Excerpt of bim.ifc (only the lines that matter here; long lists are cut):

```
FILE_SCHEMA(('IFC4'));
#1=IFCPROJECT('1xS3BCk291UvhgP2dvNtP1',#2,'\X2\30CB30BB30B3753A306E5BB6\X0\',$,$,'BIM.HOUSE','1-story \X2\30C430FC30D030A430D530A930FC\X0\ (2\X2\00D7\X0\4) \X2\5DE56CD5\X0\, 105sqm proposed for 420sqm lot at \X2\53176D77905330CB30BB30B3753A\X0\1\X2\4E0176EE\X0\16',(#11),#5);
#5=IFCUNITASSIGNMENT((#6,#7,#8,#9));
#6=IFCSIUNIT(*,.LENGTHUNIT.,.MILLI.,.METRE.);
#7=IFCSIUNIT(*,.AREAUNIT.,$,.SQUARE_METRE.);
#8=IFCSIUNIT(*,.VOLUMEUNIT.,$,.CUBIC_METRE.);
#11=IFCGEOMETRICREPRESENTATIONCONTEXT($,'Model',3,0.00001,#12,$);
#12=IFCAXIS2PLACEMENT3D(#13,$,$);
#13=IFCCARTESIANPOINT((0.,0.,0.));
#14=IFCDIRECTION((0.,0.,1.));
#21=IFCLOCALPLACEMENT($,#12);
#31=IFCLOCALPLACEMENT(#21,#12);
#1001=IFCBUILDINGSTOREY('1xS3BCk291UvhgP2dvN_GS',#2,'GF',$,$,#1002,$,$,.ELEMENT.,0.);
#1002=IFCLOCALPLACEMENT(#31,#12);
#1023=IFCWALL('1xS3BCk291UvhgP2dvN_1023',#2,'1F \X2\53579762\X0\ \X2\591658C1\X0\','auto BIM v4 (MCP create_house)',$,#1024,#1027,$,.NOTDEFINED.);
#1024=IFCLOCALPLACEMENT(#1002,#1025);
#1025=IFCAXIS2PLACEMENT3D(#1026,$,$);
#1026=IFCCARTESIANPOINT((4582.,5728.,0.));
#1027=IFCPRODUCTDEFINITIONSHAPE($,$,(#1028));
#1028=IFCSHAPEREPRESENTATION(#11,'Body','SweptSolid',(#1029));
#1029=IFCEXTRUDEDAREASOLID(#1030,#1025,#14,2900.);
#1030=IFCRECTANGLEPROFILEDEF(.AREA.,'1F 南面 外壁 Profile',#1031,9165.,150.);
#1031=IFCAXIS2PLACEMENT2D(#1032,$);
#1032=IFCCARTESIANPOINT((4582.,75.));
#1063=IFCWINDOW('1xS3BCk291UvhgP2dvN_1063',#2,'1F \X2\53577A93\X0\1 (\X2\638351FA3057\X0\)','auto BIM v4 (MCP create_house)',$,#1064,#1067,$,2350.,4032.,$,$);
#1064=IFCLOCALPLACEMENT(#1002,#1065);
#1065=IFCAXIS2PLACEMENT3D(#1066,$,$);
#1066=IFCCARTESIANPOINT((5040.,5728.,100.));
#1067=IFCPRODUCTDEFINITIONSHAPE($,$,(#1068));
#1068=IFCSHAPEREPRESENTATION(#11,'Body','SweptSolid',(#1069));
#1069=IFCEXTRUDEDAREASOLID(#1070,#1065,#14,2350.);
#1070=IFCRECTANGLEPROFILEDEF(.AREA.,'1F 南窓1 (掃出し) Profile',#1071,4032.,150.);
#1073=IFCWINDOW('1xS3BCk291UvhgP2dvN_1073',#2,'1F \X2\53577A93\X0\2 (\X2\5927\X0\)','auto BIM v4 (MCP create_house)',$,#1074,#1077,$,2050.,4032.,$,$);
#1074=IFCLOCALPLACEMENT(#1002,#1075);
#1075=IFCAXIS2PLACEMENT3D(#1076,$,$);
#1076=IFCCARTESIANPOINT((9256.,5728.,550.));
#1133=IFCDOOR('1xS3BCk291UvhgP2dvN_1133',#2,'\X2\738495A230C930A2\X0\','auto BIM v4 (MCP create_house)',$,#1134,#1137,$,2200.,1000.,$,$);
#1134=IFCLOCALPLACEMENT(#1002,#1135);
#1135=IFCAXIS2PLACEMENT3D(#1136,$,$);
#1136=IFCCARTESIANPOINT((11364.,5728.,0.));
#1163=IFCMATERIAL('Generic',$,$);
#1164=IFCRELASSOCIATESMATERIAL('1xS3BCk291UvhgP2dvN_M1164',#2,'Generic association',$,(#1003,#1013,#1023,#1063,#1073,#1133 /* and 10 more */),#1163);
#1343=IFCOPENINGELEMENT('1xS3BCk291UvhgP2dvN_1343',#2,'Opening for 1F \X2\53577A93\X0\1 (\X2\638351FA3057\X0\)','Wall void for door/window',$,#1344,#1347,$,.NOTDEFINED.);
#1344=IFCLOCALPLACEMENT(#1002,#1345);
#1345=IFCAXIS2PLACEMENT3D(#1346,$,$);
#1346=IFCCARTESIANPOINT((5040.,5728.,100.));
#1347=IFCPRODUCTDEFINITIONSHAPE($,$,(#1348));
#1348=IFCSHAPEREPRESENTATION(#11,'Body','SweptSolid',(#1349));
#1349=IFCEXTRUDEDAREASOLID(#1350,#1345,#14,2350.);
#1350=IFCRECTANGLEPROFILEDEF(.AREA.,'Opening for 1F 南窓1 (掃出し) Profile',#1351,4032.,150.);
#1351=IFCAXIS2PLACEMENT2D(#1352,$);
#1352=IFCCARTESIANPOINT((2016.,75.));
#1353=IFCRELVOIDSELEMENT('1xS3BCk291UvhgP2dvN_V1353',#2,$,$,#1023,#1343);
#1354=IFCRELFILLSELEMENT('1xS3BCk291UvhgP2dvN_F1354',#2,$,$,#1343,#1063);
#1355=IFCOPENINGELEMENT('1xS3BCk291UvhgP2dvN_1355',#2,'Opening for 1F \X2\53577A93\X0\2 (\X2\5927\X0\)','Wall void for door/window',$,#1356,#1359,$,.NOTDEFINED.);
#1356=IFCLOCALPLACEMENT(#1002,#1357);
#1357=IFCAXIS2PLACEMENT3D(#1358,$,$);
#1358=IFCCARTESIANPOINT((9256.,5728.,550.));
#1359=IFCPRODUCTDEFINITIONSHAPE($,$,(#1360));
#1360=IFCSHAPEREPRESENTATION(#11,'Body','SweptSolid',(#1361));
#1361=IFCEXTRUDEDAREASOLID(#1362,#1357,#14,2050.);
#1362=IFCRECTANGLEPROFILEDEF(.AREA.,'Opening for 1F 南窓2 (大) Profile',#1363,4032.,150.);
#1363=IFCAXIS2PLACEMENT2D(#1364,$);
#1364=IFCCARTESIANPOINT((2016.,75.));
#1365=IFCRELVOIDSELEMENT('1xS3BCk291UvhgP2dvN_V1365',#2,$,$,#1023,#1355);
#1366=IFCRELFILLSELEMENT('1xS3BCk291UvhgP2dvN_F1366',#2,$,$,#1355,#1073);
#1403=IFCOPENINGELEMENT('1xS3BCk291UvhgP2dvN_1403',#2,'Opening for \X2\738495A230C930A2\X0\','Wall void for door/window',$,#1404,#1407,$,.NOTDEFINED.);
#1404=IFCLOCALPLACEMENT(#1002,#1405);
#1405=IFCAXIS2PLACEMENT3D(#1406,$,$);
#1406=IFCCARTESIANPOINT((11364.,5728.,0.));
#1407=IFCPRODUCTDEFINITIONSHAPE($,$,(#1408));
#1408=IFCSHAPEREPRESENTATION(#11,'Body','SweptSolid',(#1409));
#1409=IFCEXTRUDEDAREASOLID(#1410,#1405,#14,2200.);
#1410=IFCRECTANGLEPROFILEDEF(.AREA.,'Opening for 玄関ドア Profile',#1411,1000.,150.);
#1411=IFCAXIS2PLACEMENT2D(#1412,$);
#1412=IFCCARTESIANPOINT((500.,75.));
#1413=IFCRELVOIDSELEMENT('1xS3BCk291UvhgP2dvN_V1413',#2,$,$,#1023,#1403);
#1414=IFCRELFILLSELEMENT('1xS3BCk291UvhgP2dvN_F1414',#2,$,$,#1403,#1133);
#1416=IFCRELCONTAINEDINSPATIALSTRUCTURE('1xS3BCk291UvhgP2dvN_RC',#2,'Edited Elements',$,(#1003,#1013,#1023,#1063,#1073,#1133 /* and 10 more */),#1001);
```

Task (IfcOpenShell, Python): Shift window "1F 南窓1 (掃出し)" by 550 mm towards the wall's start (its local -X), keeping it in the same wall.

```python
import ifcopenshell
import ifcopenshell.api.geometry
import ifcopenshell.util.placement

model = ifcopenshell.open("bim.ifc")

window = model.by_guid("1xS3BCk291UvhgP2dvN_1063")
opening = window.FillsVoids[0].RelatingOpeningElement
wall = opening.VoidsElements[0].RelatingBuildingElement

wall_matrix = ifcopenshell.util.placement.get_local_placement(wall.ObjectPlacement)
shift = wall_matrix[:3, 0] * -550.0
before = ifcopenshell.util.placement.get_local_placement(window.ObjectPlacement)[:3, 3].copy()

# The window is not placed relative to its opening, so move both.
for product in (opening, window):
    matrix = ifcopenshell.util.placement.get_local_placement(product.ObjectPlacement)
    matrix[:3, 3] += shift
    ifcopenshell.api.geometry.edit_object_placement(model, product=product, matrix=matrix, is_si=False)

after = ifcopenshell.util.placement.get_local_placement(window.ObjectPlacement)[:3, 3]
print("window moved by", (after - before).round(3) + 0.0)

model.write("bim_updated.ifc")
```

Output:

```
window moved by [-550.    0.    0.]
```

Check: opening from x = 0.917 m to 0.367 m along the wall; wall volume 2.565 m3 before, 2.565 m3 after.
